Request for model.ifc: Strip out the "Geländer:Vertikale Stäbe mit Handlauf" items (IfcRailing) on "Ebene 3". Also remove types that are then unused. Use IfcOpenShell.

First a look at what the model holds.

```python
import ifcopenshell
import ifcopenshell.util.element

model = ifcopenshell.open("model.ifc")
print(model.schema)
storey = next(s for s in model.by_type("IfcBuildingStorey") if s.Name == "Ebene 3")
railings = [e for e in ifcopenshell.util.element.get_decomposition(storey) if e.is_a("IfcRailing")]
seen = {}
for e in railings:
    element_type = ifcopenshell.util.element.get_type(e)
    name = element_type.Name if element_type not in (None, e) else None
    seen[name] = seen.get(name, 0) + 1
for name, count in sorted(seen.items(), key=str):
    print(count, "x", name)
```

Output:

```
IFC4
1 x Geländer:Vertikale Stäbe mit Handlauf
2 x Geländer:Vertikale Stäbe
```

```python
import ifcopenshell
import ifcopenshell.api.root
import ifcopenshell.util.element

model = ifcopenshell.open("model.ifc")

storey = next(s for s in model.by_type("IfcBuildingStorey") if s.Name == "Ebene 3")
railings = [e for e in ifcopenshell.util.element.get_decomposition(storey) if e.is_a("IfcRailing")]
targets = [e for e in railings if (t := ifcopenshell.util.element.get_type(e)) not in (None, e) and t.Name == "Geländer:Vertikale Stäbe mit Handlauf"]
types = {ifcopenshell.util.element.get_type(e) for e in targets} - {None, *targets}

for e in targets:
    ifcopenshell.api.root.remove_product(model, product=e)
print(len(targets), "removed")

unused = [t for t in types if not ifcopenshell.util.element.get_types(t)]
for t in unused:
    ifcopenshell.api.root.remove_product(model, product=t)
print(len(unused), "unused types removed")

model.write("model-out.ifc")
```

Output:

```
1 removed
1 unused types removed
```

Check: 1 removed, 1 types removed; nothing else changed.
